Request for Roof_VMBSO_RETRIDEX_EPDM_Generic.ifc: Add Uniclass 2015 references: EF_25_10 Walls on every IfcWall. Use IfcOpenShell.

First a look at what the model holds.

```python
import ifcopenshell

model = ifcopenshell.open("Roof_VMBSO_RETRIDEX_EPDM_Generic.ifc")
print(model.schema)
print("classifications:", [c.Name for c in model.by_type("IfcClassification")])
for ifc_class in ("IfcDoor", "IfcRoof", "IfcStair", "IfcWall", "IfcWindow"):
    print(ifc_class, len(model.by_type(ifc_class)))
```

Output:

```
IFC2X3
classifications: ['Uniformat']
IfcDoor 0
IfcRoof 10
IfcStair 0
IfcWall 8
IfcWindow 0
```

```python
import ifcopenshell
import ifcopenshell.api.classification

model = ifcopenshell.open("Roof_VMBSO_RETRIDEX_EPDM_Generic.ifc")

# IFC2X3 requires Source and Edition and has no link from the project to the system.
system = model.create_entity("IfcClassification", Source="NBS", Edition="2015", Name="Uniclass 2015")

codes = {
    "IfcWall": ("EF_25_10", "Walls"),
}
for ifc_class, (code, name) in codes.items():
    products = model.by_type(ifc_class)
    ifcopenshell.api.classification.add_reference(
        model, products=products, classification=system, identification=code, name=name
    )
    print(code, len(products))

model.write("Roof_VMBSO_RETRIDEX_EPDM_Generic_updated.ifc")
```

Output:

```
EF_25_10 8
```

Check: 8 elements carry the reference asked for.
